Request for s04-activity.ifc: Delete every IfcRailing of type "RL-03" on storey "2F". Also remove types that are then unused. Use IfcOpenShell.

First a look at what the model holds.

```python
import ifcopenshell
import ifcopenshell.util.element

model = ifcopenshell.open("s04-activity.ifc")
print(model.schema)
storey = next(s for s in model.by_type("IfcBuildingStorey") if s.Name == "2F")
railings = [e for e in ifcopenshell.util.element.get_decomposition(storey) if e.is_a("IfcRailing")]
seen = {}
for e in railings:
    element_type = ifcopenshell.util.element.get_type(e)
    name = element_type.Name if element_type not in (None, e) else None
    seen[name] = seen.get(name, 0) + 1
for name, count in sorted(seen.items(), key=str):
    print(count, "x", name)
```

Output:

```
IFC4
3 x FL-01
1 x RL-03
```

```python
import ifcopenshell
import ifcopenshell.api.root
import ifcopenshell.util.element

model = ifcopenshell.open("s04-activity.ifc")

storey = next(s for s in model.by_type("IfcBuildingStorey") if s.Name == "2F")
railings = [e for e in ifcopenshell.util.element.get_decomposition(storey) if e.is_a("IfcRailing")]
targets = [e for e in railings if (t := ifcopenshell.util.element.get_type(e)) not in (None, e) and t.Name == "RL-03"]
types = {ifcopenshell.util.element.get_type(e) for e in targets} - {None, *targets}

for e in targets:
    ifcopenshell.api.root.remove_product(model, product=e)
print(len(targets), "removed")

unused = [t for t in types if not ifcopenshell.util.element.get_types(t)]
for t in unused:
    ifcopenshell.api.root.remove_product(model, product=t)
print(len(unused), "unused types removed")

model.write("s04-activity_rev.ifc")
```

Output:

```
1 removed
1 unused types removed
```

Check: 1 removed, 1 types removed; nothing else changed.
